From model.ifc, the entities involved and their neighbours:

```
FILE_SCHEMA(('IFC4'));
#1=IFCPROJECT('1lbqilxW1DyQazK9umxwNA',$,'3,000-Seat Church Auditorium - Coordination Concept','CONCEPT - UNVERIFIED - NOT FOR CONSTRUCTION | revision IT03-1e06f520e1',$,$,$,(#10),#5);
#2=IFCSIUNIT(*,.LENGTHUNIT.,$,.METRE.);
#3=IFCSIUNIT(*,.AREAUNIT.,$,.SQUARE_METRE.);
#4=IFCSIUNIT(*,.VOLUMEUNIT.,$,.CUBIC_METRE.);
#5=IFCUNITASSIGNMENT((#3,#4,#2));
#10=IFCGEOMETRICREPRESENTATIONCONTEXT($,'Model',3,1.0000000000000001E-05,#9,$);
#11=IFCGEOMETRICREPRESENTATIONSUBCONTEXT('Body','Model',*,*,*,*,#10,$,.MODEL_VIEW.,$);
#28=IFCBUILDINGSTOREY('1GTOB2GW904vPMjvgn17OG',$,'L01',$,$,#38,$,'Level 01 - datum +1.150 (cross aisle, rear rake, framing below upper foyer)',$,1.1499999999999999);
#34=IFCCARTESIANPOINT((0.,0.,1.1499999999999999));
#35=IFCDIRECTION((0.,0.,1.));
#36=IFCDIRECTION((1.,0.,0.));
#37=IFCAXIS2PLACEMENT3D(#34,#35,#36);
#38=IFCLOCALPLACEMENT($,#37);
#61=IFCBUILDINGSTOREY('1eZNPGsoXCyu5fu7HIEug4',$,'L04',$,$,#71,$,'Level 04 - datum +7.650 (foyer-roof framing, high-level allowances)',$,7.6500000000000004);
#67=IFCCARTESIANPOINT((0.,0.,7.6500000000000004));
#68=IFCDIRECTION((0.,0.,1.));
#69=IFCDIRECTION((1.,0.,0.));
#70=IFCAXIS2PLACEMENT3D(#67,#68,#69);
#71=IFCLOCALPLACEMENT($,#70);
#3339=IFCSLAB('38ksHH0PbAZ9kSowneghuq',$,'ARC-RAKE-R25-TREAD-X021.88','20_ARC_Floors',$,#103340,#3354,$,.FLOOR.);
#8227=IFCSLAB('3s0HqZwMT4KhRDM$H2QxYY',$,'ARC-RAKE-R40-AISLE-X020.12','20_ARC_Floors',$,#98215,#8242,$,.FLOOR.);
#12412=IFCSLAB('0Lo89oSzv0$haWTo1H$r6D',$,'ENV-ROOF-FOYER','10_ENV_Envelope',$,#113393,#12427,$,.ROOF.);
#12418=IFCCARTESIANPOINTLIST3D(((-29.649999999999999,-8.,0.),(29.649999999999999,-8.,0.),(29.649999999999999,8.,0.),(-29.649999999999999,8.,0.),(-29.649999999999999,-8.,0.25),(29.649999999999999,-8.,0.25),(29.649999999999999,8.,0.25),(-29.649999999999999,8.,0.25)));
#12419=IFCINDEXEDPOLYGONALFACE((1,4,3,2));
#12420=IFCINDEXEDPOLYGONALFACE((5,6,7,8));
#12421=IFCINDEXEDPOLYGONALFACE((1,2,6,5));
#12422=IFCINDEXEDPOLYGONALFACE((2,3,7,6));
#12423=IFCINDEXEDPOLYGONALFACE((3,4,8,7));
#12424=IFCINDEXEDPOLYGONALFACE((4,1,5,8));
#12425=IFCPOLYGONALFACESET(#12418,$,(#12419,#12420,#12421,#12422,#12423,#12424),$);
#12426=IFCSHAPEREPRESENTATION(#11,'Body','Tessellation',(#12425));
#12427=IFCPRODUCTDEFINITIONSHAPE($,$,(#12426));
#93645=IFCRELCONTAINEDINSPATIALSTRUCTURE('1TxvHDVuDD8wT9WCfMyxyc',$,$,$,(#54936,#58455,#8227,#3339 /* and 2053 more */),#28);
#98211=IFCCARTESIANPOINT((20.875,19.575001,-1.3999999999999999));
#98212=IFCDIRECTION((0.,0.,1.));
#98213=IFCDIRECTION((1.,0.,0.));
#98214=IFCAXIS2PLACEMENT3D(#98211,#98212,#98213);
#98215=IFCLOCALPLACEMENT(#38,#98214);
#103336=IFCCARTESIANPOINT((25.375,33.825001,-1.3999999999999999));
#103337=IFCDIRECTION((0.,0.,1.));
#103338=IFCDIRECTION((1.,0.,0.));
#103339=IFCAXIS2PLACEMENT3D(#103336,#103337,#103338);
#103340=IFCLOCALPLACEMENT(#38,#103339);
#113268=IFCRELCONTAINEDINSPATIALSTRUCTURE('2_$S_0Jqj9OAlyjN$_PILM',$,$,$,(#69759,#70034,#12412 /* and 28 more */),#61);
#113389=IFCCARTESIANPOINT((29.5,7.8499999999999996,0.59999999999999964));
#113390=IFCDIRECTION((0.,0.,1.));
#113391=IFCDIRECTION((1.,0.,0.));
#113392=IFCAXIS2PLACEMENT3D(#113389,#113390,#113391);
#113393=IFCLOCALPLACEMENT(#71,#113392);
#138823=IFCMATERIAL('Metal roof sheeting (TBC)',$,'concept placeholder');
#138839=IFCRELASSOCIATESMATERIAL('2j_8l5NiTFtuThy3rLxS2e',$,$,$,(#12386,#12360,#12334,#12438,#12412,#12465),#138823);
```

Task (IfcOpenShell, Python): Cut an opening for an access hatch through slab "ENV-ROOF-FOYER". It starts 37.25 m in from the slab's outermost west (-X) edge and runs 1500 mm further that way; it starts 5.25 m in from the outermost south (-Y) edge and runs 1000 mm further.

```python
import numpy as np
import ifcopenshell
import ifcopenshell.api.feature
import ifcopenshell.api.geometry
import ifcopenshell.api.root
import ifcopenshell.geom
import ifcopenshell.util.placement
import ifcopenshell.util.representation
import ifcopenshell.util.shape
import ifcopenshell.util.unit

model = ifcopenshell.open("model.ifc")
unit_scale = ifcopenshell.util.unit.calculate_unit_scale(model)
settings = ifcopenshell.geom.settings()


def volume(element):
    """Net volume in cubic metres, openings subtracted."""
    shape = ifcopenshell.geom.create_shape(settings, element)
    return ifcopenshell.util.shape.get_volume(shape.geometry)


slab = model.by_guid("0Lo89oSzv0$haWTo1H$r6D")
before = volume(slab)

# Extent in the slab's own axes, in metres. The edges named are its -X and -Y sides.
slab_shape = ifcopenshell.geom.create_shape(settings, slab)
vertices = ifcopenshell.util.shape.get_vertices(slab_shape.geometry)
x_min, y_min, bottom = vertices.min(axis=0)
top = vertices[:, 2].max()

opening = ifcopenshell.api.root.create_entity(model, ifc_class="IfcOpeningElement", name="Access hatch opening", predefined_type="OPENING")
context = ifcopenshell.util.representation.get_context(model, "Model", "Body", "MODEL_VIEW")
width, depth = 1.5, 1
outline = [(0.0, 0.0), (width, 0.0), (width, depth), (0.0, depth), (0.0, 0.0)]
# Overshoot both faces by 50 mm so the cut is clean.
shape = ifcopenshell.api.geometry.add_slab_representation(
    model, context=context, depth=top - bottom + 0.1, polyline=outline
)
ifcopenshell.api.geometry.assign_representation(model, product=opening, representation=shape)

matrix = ifcopenshell.util.placement.get_local_placement(slab.ObjectPlacement)
matrix[:, 3] = matrix @ np.append(np.array([x_min + 37.25, y_min + 5.25, bottom - 0.05]) / unit_scale, 1.0)
ifcopenshell.api.geometry.edit_object_placement(model, product=opening, matrix=matrix, is_si=False)
ifcopenshell.api.feature.add_feature(model, feature=opening, element=slab)

after = volume(slab)

print(f"slab volume {before:.3f} -> {after:.3f} m3")

model.write("model_updated.ifc")
```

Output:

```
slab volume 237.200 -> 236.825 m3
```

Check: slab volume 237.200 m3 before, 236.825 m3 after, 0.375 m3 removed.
